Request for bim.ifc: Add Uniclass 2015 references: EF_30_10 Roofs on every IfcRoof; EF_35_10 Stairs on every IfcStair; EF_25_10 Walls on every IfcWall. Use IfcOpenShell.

First a look at what the model holds.

```python
import ifcopenshell

model = ifcopenshell.open("bim.ifc")
print(model.schema)
print("classifications:", [c.Name for c in model.by_type("IfcClassification")])
for ifc_class in ("IfcDoor", "IfcRoof", "IfcStair", "IfcWall", "IfcWindow"):
    print(ifc_class, len(model.by_type(ifc_class)))
```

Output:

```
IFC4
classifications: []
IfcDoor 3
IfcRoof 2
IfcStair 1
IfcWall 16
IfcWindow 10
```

```python
import ifcopenshell
import ifcopenshell.api.classification

model = ifcopenshell.open("bim.ifc")

system = ifcopenshell.api.classification.add_classification(model, classification="Uniclass 2015")

codes = {
    "IfcRoof": ("EF_30_10", "Roofs"),
    "IfcStair": ("EF_35_10", "Stairs"),
    "IfcWall": ("EF_25_10", "Walls"),
}
for ifc_class, (code, name) in codes.items():
    products = model.by_type(ifc_class)
    ifcopenshell.api.classification.add_reference(
        model, products=products, classification=system, identification=code, name=name
    )
    print(code, len(products))

model.write("bim_updated.ifc")
```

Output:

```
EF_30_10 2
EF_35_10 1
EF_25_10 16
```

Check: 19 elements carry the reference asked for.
